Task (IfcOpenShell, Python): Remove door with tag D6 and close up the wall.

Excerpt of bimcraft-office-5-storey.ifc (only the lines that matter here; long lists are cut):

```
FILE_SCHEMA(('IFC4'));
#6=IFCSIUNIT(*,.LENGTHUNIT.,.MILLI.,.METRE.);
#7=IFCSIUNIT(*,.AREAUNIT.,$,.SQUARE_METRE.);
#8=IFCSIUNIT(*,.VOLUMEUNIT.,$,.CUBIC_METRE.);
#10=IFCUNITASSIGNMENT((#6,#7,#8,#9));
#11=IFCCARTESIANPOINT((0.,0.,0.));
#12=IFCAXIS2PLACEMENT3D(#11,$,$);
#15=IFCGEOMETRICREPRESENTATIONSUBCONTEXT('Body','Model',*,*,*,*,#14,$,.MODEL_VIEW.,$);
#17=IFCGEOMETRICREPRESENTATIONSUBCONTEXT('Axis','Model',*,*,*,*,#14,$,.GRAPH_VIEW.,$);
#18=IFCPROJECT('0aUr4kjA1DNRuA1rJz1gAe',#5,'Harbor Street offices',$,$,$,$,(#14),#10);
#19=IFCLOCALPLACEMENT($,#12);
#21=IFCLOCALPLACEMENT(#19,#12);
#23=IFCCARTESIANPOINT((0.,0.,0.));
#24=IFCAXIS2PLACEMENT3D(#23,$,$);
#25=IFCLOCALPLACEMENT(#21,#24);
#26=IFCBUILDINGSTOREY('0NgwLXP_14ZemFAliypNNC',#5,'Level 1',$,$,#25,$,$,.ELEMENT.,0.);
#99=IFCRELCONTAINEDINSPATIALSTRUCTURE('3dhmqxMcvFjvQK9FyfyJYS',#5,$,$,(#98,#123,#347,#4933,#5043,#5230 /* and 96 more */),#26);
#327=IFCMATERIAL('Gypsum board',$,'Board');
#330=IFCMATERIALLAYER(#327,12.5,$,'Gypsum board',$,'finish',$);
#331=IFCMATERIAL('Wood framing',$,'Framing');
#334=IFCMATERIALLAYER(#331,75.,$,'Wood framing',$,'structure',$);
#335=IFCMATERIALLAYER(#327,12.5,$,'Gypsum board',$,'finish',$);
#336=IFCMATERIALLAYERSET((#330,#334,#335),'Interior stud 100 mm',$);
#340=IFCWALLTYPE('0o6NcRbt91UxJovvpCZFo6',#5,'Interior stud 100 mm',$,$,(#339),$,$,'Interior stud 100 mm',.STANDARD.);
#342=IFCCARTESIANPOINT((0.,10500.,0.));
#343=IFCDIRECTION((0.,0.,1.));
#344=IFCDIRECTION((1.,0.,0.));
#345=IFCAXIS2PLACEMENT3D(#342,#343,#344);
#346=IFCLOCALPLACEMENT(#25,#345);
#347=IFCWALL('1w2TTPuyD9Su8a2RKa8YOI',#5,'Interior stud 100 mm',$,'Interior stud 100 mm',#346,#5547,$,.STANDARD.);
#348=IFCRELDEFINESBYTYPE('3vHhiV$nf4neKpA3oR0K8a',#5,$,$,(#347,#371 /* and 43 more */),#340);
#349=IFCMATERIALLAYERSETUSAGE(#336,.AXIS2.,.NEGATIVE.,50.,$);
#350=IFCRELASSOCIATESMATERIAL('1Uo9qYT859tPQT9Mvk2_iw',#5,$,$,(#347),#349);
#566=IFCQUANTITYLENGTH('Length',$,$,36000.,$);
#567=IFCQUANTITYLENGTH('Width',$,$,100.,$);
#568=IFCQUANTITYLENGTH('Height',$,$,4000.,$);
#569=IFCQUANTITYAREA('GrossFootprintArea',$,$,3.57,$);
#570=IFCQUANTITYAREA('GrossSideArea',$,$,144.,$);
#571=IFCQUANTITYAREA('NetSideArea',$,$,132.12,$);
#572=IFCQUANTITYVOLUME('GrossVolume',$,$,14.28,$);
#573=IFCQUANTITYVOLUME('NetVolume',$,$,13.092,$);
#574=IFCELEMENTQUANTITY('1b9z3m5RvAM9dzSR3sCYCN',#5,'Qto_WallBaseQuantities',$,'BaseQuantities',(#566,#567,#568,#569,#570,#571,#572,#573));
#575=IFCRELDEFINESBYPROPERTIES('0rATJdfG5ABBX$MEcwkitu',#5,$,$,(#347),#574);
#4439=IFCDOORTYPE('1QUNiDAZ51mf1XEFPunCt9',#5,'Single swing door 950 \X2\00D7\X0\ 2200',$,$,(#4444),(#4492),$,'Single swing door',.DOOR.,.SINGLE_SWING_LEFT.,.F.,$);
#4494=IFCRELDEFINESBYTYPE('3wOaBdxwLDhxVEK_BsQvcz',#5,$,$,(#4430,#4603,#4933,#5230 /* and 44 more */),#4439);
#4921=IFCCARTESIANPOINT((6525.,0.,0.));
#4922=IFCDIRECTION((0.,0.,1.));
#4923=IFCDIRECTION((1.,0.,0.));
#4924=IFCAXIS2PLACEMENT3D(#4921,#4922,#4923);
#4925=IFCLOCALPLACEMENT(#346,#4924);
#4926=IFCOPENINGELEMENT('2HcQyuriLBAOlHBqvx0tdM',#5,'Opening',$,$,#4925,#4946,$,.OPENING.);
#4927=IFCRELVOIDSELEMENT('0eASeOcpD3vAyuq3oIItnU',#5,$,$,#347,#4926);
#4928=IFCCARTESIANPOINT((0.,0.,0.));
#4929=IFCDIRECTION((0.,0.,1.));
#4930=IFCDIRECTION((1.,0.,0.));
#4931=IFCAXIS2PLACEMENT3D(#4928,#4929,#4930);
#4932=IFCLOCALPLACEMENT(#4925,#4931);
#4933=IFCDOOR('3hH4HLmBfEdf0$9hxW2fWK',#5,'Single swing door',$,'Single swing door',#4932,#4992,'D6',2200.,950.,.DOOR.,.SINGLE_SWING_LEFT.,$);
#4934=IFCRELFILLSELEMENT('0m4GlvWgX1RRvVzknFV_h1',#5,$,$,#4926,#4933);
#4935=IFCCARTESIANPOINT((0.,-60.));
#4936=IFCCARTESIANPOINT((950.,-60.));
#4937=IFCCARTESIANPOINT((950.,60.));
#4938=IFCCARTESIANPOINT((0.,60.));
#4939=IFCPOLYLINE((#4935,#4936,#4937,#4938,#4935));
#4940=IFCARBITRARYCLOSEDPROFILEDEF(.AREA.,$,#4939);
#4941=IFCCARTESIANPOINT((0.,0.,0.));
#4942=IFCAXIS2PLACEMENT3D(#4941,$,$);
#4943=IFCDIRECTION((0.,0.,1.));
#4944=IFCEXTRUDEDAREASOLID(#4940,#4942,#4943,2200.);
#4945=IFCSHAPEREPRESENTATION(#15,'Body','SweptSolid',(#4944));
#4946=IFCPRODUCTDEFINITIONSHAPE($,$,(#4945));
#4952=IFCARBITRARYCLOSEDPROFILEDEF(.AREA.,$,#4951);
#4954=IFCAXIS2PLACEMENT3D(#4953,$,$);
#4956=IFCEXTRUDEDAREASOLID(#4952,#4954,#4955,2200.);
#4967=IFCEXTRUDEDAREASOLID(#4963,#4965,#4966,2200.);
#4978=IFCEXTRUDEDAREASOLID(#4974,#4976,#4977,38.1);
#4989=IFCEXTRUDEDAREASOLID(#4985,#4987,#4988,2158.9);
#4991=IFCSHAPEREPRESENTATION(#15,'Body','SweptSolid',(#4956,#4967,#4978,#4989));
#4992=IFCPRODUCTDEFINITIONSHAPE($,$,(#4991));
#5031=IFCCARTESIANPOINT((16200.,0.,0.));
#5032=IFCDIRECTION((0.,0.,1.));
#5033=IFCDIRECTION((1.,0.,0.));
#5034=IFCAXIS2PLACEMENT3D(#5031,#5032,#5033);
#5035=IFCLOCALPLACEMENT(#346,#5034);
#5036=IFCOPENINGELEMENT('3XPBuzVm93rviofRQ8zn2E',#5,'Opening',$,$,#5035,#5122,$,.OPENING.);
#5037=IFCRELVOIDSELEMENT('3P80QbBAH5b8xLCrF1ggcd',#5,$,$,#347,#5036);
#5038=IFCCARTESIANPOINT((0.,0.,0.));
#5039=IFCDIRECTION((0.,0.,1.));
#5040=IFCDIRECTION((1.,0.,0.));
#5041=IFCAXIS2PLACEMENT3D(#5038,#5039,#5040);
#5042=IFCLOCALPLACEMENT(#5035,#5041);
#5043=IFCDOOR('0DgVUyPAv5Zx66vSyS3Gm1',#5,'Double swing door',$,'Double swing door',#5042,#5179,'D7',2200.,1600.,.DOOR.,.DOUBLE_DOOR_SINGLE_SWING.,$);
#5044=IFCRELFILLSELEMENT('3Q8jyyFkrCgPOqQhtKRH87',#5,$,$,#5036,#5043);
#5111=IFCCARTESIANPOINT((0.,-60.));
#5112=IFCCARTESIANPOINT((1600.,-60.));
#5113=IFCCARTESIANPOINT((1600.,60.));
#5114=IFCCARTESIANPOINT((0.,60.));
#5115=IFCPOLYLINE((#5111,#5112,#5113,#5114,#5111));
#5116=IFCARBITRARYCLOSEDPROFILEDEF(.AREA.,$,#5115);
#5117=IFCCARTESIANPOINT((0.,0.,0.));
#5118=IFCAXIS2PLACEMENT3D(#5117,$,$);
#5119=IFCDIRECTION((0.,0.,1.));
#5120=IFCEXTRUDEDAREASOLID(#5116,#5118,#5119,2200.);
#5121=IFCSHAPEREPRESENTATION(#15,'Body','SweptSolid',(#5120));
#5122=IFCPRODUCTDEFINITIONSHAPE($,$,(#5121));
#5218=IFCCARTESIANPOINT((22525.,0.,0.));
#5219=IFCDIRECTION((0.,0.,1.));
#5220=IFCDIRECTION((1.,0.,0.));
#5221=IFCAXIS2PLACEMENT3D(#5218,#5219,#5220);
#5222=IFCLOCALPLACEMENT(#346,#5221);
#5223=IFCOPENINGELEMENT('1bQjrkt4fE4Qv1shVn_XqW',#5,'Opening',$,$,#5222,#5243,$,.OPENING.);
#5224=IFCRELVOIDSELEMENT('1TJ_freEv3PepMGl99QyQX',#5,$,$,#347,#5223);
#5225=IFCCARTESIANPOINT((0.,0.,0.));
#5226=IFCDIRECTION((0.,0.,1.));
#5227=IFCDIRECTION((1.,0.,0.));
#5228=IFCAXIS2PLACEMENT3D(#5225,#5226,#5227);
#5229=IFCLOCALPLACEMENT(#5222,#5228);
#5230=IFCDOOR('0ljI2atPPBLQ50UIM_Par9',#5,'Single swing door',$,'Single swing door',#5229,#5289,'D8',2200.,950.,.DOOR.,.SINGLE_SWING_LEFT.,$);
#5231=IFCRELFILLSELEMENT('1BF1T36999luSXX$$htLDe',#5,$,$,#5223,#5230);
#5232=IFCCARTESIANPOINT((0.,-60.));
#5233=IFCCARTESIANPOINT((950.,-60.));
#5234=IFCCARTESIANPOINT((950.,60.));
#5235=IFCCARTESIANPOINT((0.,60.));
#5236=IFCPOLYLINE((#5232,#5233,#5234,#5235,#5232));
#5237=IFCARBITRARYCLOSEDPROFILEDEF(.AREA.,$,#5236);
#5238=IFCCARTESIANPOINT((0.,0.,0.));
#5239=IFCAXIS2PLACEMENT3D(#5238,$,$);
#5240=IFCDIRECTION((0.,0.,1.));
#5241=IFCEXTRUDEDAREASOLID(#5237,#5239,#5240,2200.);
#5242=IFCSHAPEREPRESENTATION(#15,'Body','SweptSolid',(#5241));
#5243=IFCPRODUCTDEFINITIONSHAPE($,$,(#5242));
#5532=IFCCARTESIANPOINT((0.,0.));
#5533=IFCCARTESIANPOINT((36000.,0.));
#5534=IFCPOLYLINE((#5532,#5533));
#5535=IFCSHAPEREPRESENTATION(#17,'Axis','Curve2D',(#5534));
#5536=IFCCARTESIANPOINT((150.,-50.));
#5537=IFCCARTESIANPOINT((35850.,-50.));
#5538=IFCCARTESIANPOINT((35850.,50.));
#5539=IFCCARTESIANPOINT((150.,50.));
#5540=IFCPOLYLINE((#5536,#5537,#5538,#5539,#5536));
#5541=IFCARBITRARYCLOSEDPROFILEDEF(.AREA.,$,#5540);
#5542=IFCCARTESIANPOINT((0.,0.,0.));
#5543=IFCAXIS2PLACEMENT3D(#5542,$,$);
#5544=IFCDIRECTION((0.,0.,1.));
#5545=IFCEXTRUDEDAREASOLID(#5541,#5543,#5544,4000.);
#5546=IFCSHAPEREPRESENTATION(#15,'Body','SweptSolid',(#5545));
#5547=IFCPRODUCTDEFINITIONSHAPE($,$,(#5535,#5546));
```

```python
import ifcopenshell
import ifcopenshell.api.feature
import ifcopenshell.api.pset
import ifcopenshell.api.root
import ifcopenshell.geom
import ifcopenshell.util.element
import ifcopenshell.util.shape
import ifcopenshell.util.unit

model = ifcopenshell.open("bimcraft-office-5-storey.ifc")
area_scale = ifcopenshell.util.unit.calculate_unit_scale(model, "AREAUNIT")
volume_scale = ifcopenshell.util.unit.calculate_unit_scale(model, "VOLUMEUNIT")
settings = ifcopenshell.geom.settings()


def volume(element):
    """Net volume in cubic metres, openings subtracted."""
    shape = ifcopenshell.geom.create_shape(settings, element)
    return ifcopenshell.util.shape.get_volume(shape.geometry)


door = model.by_guid("3hH4HLmBfEdf0$9hxW2fWK")
opening = door.FillsVoids[0].RelatingOpeningElement
wall = opening.VoidsElements[0].RelatingBuildingElement
before = volume(wall)

ifcopenshell.api.root.remove_product(model, product=door)
ifcopenshell.api.feature.remove_feature(model, feature=opening)

after = volume(wall)
thickness = 0.1  # wall thickness in metres

# Update the wall's stored quantities.
qto = model.by_id(ifcopenshell.util.element.get_pset(wall, "Qto_WallBaseQuantities", should_inherit=False)["id"])
ifcopenshell.api.pset.edit_qto(model, qto=qto, properties={
    "NetSideArea": after / thickness / area_scale,
    "NetVolume": after / volume_scale,
})

print(f"wall volume {before:.3f} -> {after:.3f} m3")

model.write("bimcraft-office-5-storey-out.ifc")
```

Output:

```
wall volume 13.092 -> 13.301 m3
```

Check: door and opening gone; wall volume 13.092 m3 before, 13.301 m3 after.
